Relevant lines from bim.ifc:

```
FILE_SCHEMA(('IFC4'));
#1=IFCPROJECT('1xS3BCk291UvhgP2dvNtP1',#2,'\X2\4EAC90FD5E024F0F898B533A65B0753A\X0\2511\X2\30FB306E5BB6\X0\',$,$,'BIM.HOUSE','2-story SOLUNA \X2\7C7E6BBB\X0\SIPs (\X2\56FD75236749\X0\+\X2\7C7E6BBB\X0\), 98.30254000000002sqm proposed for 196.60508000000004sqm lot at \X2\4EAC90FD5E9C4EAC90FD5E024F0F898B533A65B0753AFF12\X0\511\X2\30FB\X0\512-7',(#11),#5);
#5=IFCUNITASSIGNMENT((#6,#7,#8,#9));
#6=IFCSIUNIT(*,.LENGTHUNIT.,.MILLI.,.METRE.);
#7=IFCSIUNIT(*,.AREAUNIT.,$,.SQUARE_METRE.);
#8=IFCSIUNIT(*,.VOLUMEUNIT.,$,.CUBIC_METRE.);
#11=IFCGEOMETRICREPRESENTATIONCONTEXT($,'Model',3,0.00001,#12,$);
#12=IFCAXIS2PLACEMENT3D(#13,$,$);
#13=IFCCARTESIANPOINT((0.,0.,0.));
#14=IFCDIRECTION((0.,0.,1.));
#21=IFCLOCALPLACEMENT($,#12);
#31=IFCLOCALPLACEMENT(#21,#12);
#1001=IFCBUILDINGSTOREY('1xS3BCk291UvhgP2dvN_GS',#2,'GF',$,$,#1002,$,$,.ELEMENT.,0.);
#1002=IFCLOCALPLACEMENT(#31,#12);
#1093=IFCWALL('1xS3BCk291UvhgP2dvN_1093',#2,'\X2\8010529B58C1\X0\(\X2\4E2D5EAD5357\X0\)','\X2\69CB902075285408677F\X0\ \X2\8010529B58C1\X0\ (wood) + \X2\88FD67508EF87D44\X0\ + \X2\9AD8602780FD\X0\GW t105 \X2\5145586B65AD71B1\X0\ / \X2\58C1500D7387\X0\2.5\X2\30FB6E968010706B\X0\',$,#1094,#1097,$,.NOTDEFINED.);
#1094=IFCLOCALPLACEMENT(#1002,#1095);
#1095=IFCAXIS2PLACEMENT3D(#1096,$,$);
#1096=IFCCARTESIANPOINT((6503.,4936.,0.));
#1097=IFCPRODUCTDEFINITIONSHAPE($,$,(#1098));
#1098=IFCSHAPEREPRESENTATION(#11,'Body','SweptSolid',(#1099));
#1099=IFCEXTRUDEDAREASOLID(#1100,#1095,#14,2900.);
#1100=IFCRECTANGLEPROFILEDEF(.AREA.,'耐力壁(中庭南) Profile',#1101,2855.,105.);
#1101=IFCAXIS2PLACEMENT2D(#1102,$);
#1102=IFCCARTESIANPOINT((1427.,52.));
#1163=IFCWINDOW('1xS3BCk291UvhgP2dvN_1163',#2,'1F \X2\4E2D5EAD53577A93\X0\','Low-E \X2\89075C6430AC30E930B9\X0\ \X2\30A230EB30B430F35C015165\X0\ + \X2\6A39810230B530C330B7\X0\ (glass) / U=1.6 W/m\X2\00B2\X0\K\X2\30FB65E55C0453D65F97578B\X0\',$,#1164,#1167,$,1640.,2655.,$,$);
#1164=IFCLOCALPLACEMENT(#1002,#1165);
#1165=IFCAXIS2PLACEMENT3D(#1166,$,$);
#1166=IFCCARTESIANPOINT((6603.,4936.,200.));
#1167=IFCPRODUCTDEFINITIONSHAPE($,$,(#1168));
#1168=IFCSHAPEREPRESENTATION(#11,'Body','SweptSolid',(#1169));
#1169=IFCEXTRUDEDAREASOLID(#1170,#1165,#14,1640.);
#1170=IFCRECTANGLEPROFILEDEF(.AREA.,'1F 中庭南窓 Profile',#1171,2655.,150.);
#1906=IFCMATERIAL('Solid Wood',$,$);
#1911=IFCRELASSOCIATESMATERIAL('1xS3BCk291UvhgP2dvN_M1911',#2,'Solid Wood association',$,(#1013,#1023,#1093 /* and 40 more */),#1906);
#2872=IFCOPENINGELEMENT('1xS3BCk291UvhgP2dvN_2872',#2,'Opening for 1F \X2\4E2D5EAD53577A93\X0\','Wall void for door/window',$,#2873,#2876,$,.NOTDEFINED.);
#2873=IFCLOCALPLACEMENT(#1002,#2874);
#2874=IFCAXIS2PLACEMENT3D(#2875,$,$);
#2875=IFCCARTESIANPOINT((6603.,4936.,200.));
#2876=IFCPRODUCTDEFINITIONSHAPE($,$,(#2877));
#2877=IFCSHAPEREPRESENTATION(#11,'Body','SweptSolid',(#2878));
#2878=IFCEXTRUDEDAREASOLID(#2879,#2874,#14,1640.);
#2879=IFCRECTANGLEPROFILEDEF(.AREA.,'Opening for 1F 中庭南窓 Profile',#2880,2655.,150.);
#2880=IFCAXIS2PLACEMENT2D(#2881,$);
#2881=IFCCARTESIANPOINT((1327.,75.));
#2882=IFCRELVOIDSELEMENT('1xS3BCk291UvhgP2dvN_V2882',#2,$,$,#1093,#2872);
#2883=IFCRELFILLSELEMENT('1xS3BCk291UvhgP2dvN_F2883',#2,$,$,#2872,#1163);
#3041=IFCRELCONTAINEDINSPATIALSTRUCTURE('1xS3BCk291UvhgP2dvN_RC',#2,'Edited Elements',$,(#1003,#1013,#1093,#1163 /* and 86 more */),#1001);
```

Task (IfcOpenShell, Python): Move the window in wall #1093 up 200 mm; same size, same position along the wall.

```python
import numpy as np
import ifcopenshell
import ifcopenshell.api.geometry
import ifcopenshell.util.placement
import ifcopenshell.util.unit

model = ifcopenshell.open("bim.ifc")
unit_scale = ifcopenshell.util.unit.calculate_unit_scale(model)

window = model.by_guid("1xS3BCk291UvhgP2dvN_1163")
opening = window.FillsVoids[0].RelatingOpeningElement
dz = 200.0

shift = np.array([0.0, 0.0, dz])
# The window is not placed relative to its opening, so move both.
for product in (opening, window):
    matrix = ifcopenshell.util.placement.get_local_placement(product.ObjectPlacement)
    matrix[:3, 3] += shift
    ifcopenshell.api.geometry.edit_object_placement(model, product=product, matrix=matrix, is_si=False)

print(f"moved by {dz * unit_scale:+.3f} m")

model.write("bim-out.ifc")
```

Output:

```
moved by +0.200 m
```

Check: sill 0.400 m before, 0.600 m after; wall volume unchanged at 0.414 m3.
